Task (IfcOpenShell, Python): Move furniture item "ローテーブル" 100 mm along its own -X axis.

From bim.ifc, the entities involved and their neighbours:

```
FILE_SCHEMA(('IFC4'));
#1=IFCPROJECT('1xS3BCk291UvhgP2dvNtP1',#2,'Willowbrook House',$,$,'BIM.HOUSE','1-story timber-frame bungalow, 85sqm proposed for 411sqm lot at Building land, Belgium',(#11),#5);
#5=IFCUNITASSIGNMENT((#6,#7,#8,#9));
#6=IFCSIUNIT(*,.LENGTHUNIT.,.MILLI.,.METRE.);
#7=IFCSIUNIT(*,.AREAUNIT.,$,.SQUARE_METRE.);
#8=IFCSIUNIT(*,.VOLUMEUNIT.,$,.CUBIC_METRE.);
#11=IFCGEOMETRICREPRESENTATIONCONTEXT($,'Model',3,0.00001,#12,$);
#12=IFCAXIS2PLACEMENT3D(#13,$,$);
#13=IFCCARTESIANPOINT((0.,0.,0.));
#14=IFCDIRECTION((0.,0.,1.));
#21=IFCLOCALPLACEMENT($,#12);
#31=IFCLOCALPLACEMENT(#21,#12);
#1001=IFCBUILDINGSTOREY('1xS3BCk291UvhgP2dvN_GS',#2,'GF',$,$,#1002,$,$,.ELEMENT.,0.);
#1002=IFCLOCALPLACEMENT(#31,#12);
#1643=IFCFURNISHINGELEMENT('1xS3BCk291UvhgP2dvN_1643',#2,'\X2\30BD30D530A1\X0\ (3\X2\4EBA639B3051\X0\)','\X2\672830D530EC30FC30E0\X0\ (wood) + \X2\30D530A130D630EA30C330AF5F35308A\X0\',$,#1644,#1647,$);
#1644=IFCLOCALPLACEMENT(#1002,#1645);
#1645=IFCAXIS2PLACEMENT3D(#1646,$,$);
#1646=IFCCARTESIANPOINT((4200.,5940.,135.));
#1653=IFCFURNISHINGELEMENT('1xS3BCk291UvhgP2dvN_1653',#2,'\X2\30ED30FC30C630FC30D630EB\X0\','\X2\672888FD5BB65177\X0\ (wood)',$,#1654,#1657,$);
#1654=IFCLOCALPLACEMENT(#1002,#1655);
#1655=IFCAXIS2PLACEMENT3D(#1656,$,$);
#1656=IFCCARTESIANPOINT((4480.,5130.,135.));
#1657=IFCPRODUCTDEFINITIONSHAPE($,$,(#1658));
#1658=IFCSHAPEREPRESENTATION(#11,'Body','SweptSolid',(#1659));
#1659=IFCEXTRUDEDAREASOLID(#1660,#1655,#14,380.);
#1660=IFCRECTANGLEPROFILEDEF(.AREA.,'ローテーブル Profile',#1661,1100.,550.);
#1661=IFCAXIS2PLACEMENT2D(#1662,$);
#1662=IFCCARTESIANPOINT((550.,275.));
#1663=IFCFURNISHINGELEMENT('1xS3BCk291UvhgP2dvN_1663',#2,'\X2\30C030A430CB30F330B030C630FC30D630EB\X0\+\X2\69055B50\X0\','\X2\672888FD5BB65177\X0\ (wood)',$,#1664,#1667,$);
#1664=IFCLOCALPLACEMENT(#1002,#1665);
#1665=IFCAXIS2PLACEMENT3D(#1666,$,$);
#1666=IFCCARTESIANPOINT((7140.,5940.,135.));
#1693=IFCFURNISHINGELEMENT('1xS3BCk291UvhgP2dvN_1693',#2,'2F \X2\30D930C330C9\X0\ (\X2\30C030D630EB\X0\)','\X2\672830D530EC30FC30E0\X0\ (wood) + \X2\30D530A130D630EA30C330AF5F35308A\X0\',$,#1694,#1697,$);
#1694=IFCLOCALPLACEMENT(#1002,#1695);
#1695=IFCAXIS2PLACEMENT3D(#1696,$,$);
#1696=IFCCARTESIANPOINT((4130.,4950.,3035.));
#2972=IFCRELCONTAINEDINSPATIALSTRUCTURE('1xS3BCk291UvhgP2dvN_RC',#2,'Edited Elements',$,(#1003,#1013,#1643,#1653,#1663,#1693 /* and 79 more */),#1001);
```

```python
import ifcopenshell
import ifcopenshell.api.geometry
import ifcopenshell.util.placement

model = ifcopenshell.open("bim.ifc")

item = model.by_id(1653)
matrix = ifcopenshell.util.placement.get_local_placement(item.ObjectPlacement)
matrix[:3, 3] -= matrix[:3, 0] * 100.0
ifcopenshell.api.geometry.edit_object_placement(model, product=item, matrix=matrix, is_si=False)

print(ifcopenshell.util.placement.get_local_placement(item.ObjectPlacement).round(3) + 0.0)

model.write("bim_updated.ifc")
```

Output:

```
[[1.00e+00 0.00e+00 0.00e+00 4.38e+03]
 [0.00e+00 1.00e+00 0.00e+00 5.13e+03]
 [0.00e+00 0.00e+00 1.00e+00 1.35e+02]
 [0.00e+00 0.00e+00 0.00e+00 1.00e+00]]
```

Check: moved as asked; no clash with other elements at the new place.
